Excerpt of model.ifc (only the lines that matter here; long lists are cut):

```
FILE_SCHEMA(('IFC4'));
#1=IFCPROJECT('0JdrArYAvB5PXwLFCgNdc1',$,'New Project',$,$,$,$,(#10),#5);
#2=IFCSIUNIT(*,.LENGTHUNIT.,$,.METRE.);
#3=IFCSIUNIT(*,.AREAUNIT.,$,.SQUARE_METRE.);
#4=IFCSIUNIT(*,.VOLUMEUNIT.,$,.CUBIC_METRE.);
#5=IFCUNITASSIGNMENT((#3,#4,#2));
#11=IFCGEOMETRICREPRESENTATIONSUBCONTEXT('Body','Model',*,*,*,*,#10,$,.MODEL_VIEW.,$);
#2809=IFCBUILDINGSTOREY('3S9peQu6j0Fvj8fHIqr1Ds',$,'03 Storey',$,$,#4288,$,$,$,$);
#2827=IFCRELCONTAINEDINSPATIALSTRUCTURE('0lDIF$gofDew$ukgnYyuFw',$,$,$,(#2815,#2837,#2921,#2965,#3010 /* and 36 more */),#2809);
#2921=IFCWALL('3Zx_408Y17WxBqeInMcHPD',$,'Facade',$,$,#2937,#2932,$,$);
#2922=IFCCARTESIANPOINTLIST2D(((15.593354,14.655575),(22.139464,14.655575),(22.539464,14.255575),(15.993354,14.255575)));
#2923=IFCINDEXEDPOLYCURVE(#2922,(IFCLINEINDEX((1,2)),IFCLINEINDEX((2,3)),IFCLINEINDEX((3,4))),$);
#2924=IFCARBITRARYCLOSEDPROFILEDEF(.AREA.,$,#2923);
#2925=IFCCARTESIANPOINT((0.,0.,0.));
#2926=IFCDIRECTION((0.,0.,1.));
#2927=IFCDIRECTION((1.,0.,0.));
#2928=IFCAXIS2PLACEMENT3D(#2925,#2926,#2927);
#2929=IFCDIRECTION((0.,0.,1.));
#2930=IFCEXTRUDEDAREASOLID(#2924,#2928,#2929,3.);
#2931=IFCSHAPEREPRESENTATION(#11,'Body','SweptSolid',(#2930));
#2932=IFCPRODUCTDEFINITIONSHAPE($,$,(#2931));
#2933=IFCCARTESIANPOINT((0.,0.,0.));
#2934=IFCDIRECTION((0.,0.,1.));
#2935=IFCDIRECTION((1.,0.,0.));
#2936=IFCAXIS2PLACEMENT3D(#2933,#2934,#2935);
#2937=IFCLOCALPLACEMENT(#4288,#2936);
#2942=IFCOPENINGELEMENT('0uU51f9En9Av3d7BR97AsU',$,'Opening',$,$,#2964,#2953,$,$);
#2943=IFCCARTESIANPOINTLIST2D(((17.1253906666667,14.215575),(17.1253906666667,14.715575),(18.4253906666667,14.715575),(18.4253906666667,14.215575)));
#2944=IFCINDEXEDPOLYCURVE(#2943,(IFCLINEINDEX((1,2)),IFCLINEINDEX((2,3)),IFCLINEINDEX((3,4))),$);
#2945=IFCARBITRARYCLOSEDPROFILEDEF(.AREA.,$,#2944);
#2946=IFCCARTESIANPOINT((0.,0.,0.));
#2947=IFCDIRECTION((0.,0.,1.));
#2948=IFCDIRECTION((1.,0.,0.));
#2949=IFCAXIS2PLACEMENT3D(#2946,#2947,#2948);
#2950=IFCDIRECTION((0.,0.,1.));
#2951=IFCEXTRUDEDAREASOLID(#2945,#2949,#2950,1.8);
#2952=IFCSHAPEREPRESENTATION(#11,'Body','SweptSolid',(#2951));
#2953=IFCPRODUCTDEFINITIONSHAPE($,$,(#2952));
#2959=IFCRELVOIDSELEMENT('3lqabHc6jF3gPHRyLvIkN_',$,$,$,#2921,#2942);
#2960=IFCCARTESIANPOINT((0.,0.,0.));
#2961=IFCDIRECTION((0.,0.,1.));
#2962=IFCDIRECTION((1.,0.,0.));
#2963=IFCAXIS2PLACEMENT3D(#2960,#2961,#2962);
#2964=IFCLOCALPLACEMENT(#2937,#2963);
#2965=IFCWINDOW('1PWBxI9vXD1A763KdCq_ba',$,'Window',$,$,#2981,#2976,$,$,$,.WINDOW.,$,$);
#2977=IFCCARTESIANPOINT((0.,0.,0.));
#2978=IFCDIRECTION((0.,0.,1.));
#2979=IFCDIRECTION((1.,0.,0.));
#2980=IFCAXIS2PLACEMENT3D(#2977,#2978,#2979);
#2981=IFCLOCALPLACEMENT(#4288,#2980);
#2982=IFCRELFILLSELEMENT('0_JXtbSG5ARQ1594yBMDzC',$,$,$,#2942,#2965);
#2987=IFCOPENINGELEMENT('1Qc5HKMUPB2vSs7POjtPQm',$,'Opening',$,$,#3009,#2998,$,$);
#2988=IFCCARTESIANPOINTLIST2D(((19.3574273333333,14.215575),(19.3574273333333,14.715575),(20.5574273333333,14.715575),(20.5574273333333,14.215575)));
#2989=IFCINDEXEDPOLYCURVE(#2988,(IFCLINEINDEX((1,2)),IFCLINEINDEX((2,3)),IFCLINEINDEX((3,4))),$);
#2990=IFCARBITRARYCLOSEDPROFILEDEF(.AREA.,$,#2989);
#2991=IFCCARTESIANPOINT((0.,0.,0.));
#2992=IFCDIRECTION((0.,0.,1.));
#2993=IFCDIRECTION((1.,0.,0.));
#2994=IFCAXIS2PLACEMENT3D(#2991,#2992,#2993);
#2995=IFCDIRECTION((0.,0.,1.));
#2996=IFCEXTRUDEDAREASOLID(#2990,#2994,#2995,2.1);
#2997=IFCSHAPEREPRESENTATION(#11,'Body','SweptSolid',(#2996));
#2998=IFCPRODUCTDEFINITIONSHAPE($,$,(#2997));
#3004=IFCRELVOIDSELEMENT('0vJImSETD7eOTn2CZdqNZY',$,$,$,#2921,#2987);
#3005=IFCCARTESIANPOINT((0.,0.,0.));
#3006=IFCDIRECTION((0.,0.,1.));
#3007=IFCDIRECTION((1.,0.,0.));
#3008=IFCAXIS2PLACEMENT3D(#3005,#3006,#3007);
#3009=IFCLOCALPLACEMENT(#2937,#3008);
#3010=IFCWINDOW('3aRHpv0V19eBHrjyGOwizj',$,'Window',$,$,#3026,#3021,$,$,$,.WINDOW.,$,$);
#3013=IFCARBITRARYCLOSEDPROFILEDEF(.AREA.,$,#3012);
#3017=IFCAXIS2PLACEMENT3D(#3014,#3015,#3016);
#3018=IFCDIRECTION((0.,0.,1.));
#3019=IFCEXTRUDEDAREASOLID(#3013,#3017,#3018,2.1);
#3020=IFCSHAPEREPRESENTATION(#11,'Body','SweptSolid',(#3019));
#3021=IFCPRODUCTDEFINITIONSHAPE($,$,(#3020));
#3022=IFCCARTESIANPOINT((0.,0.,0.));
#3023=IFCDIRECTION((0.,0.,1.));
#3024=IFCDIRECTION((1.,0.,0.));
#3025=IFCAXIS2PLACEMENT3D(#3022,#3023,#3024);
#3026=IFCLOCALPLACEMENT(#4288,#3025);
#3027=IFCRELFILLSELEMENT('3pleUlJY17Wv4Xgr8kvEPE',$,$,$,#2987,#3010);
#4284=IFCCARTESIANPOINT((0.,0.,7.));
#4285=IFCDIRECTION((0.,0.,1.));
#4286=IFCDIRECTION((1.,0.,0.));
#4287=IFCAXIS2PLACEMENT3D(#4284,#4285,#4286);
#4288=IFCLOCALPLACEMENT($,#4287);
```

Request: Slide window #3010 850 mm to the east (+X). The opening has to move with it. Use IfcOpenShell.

```python
import ifcopenshell
import ifcopenshell.api.geometry
import ifcopenshell.util.placement

model = ifcopenshell.open("model.ifc")

window = model.by_guid("3aRHpv0V19eBHrjyGOwizj")
opening = window.FillsVoids[0].RelatingOpeningElement
wall = opening.VoidsElements[0].RelatingBuildingElement

wall_matrix = ifcopenshell.util.placement.get_local_placement(wall.ObjectPlacement)
shift = wall_matrix[:3, 0] * 0.85
before = ifcopenshell.util.placement.get_local_placement(window.ObjectPlacement)[:3, 3].copy()

# The window is not placed relative to its opening, so move both.
for product in (opening, window):
    matrix = ifcopenshell.util.placement.get_local_placement(product.ObjectPlacement)
    matrix[:3, 3] += shift
    ifcopenshell.api.geometry.edit_object_placement(model, product=product, matrix=matrix, is_si=False)

after = ifcopenshell.util.placement.get_local_placement(window.ObjectPlacement)[:3, 3]
print("window moved by", (after - before).round(3) + 0.0)

model.write("model_edited.ifc")
```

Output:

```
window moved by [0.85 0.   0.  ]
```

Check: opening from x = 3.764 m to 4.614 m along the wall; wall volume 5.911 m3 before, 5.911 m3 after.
